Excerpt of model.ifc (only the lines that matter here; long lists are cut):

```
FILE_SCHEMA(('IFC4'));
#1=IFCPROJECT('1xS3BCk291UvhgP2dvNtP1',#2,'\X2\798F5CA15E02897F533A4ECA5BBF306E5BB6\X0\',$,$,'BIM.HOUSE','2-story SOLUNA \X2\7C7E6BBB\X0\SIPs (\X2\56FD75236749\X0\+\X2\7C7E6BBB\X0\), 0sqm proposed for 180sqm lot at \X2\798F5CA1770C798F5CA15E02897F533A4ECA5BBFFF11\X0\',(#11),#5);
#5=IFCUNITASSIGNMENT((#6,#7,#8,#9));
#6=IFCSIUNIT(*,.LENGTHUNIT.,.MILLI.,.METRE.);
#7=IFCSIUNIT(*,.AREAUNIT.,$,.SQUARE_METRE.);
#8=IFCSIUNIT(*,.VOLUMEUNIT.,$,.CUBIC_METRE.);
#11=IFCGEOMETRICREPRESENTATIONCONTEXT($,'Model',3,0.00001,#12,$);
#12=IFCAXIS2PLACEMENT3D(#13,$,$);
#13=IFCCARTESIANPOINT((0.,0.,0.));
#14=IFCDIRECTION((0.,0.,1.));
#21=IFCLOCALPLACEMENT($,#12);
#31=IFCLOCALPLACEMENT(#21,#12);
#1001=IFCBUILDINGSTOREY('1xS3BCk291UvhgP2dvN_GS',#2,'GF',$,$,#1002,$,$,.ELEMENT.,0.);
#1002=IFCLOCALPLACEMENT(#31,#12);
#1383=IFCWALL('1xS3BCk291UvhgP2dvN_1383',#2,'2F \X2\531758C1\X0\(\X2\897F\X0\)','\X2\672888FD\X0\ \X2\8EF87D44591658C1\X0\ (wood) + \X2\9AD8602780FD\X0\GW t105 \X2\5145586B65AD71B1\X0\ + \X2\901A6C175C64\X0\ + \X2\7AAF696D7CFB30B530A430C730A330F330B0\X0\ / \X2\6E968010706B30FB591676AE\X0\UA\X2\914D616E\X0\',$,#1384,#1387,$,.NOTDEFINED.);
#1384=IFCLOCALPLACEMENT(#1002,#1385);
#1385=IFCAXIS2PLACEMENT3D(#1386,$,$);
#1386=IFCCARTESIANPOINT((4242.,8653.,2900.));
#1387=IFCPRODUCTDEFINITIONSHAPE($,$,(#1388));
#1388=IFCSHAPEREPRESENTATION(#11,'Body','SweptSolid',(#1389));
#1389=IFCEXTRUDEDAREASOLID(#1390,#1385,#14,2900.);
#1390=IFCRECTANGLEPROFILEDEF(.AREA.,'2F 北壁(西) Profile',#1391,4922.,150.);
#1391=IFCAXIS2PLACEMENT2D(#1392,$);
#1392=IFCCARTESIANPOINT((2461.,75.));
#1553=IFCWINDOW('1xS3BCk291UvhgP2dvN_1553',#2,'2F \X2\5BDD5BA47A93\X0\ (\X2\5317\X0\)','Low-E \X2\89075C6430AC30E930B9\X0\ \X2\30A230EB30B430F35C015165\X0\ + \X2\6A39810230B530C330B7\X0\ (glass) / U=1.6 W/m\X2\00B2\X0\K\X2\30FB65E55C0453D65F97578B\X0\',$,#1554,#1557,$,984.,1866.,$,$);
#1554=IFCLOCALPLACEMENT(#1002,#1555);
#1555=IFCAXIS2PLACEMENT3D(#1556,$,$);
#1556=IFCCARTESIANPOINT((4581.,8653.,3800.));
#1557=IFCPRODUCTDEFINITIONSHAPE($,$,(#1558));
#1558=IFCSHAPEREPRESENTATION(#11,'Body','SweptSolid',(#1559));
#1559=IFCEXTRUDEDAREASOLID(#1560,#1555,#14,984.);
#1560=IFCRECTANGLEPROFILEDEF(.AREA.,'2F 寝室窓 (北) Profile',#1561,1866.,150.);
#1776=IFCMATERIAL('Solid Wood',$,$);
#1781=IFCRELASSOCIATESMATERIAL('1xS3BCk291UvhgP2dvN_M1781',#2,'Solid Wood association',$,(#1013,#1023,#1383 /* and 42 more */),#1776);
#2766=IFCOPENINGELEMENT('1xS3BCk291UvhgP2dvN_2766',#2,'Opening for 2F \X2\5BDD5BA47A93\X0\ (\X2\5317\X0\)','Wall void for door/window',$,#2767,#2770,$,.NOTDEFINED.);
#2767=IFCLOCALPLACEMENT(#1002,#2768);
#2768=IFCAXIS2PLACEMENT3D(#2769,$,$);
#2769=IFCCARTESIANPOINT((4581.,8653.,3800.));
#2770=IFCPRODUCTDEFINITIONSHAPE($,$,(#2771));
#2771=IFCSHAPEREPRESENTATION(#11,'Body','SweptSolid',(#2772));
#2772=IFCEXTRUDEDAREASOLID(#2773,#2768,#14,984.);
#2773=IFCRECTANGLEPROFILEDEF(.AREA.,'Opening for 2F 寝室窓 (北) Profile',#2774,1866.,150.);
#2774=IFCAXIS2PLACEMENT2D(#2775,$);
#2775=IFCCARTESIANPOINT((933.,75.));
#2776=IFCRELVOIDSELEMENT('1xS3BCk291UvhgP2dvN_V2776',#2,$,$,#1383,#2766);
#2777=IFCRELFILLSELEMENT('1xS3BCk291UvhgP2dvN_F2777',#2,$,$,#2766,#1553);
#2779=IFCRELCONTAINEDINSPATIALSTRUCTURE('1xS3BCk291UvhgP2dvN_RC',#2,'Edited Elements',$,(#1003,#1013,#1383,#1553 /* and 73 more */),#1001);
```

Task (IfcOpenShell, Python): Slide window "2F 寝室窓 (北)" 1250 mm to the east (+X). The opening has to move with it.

```python
import ifcopenshell
import ifcopenshell.api.geometry
import ifcopenshell.util.placement
import ifcopenshell.util.unit

model = ifcopenshell.open("model.ifc")
unit_scale = ifcopenshell.util.unit.calculate_unit_scale(model)

window = model.by_guid("1xS3BCk291UvhgP2dvN_1553")
opening = window.FillsVoids[0].RelatingOpeningElement
wall = opening.VoidsElements[0].RelatingBuildingElement

wall_matrix = ifcopenshell.util.placement.get_local_placement(wall.ObjectPlacement)
shift = wall_matrix[:3, 0] * 1.25 / unit_scale
before = ifcopenshell.util.placement.get_local_placement(window.ObjectPlacement)[:3, 3].copy()

# The window is not placed relative to its opening, so move both.
for product in (opening, window):
    matrix = ifcopenshell.util.placement.get_local_placement(product.ObjectPlacement)
    matrix[:3, 3] += shift
    ifcopenshell.api.geometry.edit_object_placement(model, product=product, matrix=matrix, is_si=False)

after = ifcopenshell.util.placement.get_local_placement(window.ObjectPlacement)[:3, 3]
print("window moved by", (after - before).round(3) + 0.0)

model.write("model_updated.ifc")
```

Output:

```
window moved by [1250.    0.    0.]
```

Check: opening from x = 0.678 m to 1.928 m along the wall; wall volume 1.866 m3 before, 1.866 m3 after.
